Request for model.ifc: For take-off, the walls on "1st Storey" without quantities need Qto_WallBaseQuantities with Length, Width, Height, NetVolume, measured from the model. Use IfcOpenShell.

First a look at what the model holds.

```python
import ifcopenshell
import ifcopenshell.util.element
import ifcopenshell.util.unit

model = ifcopenshell.open("model.ifc")
print(model.schema)
for unit_type in ("LENGTHUNIT", "AREAUNIT", "VOLUMEUNIT"):
    print(unit_type, ifcopenshell.util.unit.calculate_unit_scale(model, unit_type))
storey = next(s for s in model.by_type("IfcBuildingStorey") if s.Name == "1st Storey")
walls = [e for e in ifcopenshell.util.element.get_decomposition(storey) if e.is_a("IfcWall")]
for e in sorted(walls, key=lambda e: e.id()):
    print(e.id(), e.is_a(), e.Name, list(ifcopenshell.util.element.get_psets(e, qtos_only=True)), sep=" | ")
```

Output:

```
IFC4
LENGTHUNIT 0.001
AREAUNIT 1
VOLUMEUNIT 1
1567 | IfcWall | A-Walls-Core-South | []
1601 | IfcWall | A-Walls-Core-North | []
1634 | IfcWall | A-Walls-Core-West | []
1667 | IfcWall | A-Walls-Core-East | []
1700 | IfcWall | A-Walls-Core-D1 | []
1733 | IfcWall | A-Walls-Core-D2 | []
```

```python
import ifcopenshell
import ifcopenshell.api.pset
import ifcopenshell.geom
import ifcopenshell.util.element
import ifcopenshell.util.shape
import ifcopenshell.util.unit

model = ifcopenshell.open("model.ifc")
unit_scale = ifcopenshell.util.unit.calculate_unit_scale(model)
volume_scale = ifcopenshell.util.unit.calculate_unit_scale(model, "VOLUMEUNIT")
settings = ifcopenshell.geom.settings()

storey = next(s for s in model.by_type("IfcBuildingStorey") if s.Name == "1st Storey")
walls = [e for e in ifcopenshell.util.element.get_decomposition(storey) if e.is_a("IfcWall")]

for e in sorted(walls, key=lambda e: e.id()):
    if ifcopenshell.util.element.get_psets(e, qtos_only=True, should_inherit=False):
        continue
    # Geometry comes back in metres, in the element's own axes.
    shape = ifcopenshell.geom.create_shape(settings, e)
    values = {
        "Length": ifcopenshell.util.shape.get_x(shape.geometry) / unit_scale,
        "Width": ifcopenshell.util.shape.get_y(shape.geometry) / unit_scale,
        "Height": ifcopenshell.util.shape.get_z(shape.geometry) / unit_scale,
        "NetVolume": ifcopenshell.util.shape.get_volume(shape.geometry) / volume_scale,
    }
    qto = ifcopenshell.api.pset.add_qto(model, product=e, name="Qto_WallBaseQuantities")
    ifcopenshell.api.pset.edit_qto(model, qto=qto, properties=values)
    print(e.id(), {k: round(v, 3) for k, v in values.items()})

model.write("model-out.ifc")
```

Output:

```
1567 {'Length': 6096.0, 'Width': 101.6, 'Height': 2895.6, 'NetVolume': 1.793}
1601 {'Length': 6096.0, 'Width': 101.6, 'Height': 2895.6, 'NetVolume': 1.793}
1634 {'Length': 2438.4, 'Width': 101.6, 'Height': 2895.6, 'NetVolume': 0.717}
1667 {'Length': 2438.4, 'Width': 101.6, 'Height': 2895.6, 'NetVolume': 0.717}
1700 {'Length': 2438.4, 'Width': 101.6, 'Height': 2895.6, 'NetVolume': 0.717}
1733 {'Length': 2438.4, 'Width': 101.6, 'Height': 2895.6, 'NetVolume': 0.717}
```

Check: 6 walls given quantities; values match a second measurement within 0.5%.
